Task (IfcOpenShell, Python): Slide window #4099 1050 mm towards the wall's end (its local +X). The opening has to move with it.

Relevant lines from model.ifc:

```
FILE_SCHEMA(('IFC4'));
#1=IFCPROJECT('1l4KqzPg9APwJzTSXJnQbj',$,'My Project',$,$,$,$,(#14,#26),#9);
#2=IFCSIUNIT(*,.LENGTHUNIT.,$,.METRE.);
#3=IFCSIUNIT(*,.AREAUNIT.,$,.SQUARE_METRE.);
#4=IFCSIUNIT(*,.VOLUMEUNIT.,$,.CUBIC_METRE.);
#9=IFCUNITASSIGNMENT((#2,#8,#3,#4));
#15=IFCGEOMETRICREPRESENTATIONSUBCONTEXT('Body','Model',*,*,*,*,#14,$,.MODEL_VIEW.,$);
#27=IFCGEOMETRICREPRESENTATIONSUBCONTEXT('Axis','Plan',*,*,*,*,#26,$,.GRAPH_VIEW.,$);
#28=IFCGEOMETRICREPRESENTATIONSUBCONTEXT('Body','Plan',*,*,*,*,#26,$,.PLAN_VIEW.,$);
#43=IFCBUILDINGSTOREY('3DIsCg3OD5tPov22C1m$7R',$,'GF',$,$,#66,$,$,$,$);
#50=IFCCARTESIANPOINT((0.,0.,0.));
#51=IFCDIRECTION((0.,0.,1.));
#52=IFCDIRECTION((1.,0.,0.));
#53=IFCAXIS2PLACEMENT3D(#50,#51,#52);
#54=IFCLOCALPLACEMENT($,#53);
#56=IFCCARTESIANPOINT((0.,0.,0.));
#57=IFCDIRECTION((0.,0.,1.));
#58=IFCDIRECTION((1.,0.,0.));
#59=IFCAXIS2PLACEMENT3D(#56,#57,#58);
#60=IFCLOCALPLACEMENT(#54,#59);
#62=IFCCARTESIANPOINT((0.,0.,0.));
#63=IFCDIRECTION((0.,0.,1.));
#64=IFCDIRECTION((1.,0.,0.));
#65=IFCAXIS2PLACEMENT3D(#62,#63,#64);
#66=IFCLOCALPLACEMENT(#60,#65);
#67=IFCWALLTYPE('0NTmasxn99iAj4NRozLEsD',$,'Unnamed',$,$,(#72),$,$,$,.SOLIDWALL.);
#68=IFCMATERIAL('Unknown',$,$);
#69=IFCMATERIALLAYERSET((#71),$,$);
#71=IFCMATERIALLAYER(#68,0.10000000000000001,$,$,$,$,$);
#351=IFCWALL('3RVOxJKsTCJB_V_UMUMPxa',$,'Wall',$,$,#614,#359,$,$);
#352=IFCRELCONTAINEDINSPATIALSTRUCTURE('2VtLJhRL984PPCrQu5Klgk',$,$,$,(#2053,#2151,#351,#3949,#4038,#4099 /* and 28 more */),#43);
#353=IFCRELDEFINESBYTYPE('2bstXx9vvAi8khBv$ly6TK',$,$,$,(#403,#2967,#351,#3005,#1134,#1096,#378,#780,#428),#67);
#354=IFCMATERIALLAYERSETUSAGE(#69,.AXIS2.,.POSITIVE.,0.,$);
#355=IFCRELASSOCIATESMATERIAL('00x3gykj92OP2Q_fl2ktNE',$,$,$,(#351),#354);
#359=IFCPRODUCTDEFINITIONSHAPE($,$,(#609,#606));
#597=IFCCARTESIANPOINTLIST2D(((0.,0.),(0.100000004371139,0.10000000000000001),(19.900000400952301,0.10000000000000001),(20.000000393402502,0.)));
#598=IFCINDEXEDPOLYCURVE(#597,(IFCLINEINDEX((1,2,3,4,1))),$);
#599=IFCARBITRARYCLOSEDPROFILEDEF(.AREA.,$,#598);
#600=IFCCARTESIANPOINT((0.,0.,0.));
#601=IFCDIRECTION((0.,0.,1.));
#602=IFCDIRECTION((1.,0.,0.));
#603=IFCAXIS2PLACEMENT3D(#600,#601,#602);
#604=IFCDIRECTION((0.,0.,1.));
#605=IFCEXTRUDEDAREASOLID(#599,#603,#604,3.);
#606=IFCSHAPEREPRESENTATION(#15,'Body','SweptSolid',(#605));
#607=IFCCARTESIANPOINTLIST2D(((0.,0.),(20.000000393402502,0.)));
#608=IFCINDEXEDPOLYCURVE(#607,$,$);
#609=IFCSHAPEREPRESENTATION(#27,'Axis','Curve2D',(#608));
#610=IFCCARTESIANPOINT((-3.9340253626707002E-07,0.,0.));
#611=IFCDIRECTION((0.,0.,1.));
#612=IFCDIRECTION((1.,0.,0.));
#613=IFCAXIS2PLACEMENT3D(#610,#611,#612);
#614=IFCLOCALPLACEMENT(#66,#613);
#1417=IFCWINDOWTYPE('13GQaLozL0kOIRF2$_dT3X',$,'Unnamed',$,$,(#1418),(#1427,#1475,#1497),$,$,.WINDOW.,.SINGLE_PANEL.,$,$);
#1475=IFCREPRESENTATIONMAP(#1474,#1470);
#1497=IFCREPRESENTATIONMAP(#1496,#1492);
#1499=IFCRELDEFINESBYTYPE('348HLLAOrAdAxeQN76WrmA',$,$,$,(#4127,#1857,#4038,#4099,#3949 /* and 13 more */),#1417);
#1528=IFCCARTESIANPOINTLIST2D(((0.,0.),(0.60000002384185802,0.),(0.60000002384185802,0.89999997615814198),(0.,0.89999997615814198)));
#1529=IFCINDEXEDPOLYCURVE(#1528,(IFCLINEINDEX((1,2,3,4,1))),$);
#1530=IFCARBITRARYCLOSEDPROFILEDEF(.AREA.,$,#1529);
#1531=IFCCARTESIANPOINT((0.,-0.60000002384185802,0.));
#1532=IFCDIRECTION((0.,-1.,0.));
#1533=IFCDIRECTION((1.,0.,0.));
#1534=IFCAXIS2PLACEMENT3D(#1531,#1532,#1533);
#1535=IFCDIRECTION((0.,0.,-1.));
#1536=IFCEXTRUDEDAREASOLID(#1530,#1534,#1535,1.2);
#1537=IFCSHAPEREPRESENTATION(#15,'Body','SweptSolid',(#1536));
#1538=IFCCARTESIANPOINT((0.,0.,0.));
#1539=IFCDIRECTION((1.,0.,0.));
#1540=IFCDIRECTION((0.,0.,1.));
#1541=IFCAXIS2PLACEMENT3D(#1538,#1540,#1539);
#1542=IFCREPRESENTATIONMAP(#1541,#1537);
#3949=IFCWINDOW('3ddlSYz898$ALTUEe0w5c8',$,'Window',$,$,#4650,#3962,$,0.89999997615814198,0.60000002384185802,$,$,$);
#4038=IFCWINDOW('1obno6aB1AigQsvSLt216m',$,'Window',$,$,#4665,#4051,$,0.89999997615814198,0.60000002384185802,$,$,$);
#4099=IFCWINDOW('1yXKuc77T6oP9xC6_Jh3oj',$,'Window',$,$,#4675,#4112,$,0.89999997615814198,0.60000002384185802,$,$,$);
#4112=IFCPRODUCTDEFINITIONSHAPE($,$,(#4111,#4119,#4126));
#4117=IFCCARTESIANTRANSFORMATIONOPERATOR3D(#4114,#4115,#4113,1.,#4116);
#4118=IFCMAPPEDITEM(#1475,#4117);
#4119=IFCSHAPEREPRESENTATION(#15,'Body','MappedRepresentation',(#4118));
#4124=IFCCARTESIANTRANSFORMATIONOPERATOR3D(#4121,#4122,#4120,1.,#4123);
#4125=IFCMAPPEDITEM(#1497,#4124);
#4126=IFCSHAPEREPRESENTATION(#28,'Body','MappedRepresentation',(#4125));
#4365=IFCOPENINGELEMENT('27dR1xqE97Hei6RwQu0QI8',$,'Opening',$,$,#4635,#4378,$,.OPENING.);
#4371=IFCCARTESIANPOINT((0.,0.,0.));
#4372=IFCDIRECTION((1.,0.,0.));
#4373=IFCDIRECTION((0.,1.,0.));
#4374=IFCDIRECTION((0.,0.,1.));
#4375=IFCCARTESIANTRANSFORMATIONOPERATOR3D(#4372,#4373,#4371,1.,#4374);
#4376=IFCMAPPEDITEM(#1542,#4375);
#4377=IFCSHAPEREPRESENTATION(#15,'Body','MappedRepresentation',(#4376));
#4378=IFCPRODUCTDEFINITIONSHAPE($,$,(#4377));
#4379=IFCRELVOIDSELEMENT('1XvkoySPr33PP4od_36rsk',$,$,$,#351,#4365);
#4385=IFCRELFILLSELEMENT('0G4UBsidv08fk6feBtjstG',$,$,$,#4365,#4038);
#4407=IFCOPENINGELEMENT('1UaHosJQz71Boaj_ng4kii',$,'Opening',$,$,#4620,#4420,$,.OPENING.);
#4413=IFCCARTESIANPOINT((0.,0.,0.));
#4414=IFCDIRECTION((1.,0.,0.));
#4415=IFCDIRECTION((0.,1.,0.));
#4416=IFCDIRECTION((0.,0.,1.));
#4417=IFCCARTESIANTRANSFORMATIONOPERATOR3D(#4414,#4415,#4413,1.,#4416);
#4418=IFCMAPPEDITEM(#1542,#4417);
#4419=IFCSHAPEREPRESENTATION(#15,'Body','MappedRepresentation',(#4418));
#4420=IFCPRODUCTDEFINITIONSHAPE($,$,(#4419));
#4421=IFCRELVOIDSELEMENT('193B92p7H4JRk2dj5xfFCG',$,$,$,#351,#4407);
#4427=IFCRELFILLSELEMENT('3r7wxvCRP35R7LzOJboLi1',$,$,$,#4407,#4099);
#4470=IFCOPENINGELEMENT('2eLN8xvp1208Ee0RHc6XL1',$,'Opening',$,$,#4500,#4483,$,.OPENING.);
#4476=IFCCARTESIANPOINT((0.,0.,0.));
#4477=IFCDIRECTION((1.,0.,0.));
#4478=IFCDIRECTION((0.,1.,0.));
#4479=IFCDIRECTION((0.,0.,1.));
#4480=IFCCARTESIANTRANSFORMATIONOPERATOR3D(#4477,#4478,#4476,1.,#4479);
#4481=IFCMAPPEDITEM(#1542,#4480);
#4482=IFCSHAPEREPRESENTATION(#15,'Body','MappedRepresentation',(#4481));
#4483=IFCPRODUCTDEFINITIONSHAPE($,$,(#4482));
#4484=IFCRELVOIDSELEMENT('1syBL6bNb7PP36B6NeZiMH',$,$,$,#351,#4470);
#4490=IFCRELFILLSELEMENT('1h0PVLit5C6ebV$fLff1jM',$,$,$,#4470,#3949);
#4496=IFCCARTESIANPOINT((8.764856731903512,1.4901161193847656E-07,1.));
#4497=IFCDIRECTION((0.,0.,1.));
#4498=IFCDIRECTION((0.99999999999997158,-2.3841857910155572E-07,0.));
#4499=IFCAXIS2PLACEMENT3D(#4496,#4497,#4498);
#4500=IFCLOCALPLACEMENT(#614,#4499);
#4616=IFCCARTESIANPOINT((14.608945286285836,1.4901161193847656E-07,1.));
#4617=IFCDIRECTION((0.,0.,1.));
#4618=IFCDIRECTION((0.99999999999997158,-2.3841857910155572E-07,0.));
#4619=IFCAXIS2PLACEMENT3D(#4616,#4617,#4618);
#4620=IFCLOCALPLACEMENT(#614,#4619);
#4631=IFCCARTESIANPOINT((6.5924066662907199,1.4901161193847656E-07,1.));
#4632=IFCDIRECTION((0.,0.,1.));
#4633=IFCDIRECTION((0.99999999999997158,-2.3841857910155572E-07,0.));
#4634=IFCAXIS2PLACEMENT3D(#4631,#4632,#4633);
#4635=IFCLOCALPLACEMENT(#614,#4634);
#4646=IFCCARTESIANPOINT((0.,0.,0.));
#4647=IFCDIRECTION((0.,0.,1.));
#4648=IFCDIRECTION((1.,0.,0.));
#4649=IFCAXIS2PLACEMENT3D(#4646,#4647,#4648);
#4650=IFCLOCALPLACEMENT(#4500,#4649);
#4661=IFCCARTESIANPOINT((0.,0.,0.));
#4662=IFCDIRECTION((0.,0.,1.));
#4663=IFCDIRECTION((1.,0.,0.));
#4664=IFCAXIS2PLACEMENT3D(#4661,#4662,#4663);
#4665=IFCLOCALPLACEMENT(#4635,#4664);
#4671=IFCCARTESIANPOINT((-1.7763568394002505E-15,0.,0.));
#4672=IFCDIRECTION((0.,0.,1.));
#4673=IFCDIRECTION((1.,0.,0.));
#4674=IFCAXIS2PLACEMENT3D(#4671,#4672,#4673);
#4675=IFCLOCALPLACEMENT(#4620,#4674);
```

```python
import ifcopenshell
import ifcopenshell.api.geometry
import ifcopenshell.util.placement
import ifcopenshell.util.unit

model = ifcopenshell.open("model.ifc")
unit_scale = ifcopenshell.util.unit.calculate_unit_scale(model)

window = model.by_guid("1yXKuc77T6oP9xC6_Jh3oj")
opening = window.FillsVoids[0].RelatingOpeningElement
wall = opening.VoidsElements[0].RelatingBuildingElement

wall_matrix = ifcopenshell.util.placement.get_local_placement(wall.ObjectPlacement)
shift = wall_matrix[:3, 0] * 1.05 / unit_scale
before = ifcopenshell.util.placement.get_local_placement(window.ObjectPlacement)[:3, 3].copy()

# The window is placed relative to its opening, so it follows when the opening moves.
matrix = ifcopenshell.util.placement.get_local_placement(opening.ObjectPlacement)
matrix[:3, 3] += shift
ifcopenshell.api.geometry.edit_object_placement(
    model, product=opening, matrix=matrix, is_si=False, should_transform_children=True
)

after = ifcopenshell.util.placement.get_local_placement(window.ObjectPlacement)[:3, 3]
print("window moved by", (after - before).round(3) + 0.0)

model.write("model_rev.ifc")
```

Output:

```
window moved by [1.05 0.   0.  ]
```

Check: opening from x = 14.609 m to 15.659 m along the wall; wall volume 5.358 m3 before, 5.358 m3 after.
